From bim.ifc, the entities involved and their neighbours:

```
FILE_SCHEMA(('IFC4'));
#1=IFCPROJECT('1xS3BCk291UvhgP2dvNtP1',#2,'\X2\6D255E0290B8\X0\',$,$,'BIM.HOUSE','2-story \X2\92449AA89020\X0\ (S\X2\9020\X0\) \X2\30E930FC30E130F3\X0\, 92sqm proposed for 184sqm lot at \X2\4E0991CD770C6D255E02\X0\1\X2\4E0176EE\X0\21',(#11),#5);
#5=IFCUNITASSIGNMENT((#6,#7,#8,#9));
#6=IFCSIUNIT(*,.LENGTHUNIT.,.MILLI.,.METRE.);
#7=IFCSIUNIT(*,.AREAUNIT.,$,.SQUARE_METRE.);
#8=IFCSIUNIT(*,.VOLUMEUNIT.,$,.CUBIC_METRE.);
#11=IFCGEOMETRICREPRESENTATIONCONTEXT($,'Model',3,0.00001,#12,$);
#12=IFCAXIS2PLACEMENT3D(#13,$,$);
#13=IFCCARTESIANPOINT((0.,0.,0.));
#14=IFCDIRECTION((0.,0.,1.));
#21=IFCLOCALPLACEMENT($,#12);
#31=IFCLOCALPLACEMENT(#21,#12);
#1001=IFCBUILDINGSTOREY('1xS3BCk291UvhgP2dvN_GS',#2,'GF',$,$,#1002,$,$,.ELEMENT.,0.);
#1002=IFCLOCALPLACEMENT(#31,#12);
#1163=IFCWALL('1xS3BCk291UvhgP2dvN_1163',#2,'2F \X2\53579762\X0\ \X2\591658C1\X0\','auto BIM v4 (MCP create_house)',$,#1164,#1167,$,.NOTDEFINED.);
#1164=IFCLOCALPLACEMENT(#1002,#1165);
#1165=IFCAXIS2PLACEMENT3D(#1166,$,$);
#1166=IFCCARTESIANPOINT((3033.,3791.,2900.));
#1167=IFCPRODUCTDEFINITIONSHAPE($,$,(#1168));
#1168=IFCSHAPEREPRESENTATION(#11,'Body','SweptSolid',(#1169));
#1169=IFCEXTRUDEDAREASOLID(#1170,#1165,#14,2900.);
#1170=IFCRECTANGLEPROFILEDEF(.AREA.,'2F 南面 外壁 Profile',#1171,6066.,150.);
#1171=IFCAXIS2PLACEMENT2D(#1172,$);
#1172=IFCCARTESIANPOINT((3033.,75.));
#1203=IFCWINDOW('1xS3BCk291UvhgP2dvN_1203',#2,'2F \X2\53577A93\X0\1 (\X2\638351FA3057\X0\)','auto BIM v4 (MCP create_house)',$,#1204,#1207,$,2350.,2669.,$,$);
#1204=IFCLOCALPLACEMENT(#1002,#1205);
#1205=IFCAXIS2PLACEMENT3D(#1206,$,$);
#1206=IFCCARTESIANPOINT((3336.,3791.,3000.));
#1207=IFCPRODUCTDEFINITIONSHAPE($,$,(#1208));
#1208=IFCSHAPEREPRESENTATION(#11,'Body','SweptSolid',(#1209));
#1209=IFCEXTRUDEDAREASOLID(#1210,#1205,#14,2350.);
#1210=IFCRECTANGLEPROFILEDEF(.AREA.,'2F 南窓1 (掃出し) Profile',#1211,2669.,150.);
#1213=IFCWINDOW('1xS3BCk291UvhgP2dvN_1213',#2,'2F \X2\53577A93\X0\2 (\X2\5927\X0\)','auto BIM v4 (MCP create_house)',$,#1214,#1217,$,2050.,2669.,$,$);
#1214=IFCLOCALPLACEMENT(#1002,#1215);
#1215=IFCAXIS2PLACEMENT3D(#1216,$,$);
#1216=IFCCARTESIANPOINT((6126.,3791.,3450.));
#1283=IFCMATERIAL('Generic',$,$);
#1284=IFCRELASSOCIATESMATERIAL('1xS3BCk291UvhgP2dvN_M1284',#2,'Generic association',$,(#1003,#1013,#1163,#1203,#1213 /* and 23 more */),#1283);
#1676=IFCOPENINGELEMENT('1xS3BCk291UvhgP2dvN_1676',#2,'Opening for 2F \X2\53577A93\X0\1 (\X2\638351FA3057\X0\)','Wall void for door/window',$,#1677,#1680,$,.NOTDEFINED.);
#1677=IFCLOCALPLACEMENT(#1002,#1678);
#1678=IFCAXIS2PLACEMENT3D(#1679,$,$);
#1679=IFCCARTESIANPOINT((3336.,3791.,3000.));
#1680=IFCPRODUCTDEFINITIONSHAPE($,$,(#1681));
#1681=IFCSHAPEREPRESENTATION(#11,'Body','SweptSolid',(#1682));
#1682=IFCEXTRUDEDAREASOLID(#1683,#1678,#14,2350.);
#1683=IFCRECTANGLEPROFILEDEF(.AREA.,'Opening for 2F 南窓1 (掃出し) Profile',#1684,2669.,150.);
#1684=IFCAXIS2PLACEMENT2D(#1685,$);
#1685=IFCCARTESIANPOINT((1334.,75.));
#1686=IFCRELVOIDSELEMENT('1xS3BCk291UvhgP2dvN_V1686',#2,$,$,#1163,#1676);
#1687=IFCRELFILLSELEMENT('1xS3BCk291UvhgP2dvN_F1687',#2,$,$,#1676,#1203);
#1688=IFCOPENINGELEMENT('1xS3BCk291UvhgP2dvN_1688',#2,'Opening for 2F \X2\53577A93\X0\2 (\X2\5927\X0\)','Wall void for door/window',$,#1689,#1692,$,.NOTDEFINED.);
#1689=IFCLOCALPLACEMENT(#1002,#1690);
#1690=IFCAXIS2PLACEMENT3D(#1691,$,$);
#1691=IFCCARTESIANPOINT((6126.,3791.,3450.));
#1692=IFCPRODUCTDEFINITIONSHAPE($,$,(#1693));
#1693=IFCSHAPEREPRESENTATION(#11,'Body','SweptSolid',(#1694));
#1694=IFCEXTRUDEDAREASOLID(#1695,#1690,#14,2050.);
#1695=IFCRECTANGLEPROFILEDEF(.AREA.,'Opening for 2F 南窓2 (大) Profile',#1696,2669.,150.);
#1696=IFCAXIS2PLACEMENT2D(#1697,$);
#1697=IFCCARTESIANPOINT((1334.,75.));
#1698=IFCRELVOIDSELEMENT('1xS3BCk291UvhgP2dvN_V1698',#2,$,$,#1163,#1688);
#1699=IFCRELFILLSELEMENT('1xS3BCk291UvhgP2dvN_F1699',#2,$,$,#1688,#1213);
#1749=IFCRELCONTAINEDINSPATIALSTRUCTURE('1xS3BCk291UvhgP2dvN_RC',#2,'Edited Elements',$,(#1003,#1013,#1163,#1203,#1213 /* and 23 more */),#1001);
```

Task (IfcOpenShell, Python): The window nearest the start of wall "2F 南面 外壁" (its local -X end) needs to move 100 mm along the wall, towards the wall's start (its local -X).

```python
import ifcopenshell
import ifcopenshell.api.geometry
import ifcopenshell.util.placement
import ifcopenshell.util.unit

model = ifcopenshell.open("bim.ifc")
unit_scale = ifcopenshell.util.unit.calculate_unit_scale(model)

window = model.by_guid("1xS3BCk291UvhgP2dvN_1203")
opening = window.FillsVoids[0].RelatingOpeningElement
wall = opening.VoidsElements[0].RelatingBuildingElement

wall_matrix = ifcopenshell.util.placement.get_local_placement(wall.ObjectPlacement)
shift = wall_matrix[:3, 0] * -0.1 / unit_scale
before = ifcopenshell.util.placement.get_local_placement(window.ObjectPlacement)[:3, 3].copy()

# The window is not placed relative to its opening, so move both.
for product in (opening, window):
    matrix = ifcopenshell.util.placement.get_local_placement(product.ObjectPlacement)
    matrix[:3, 3] += shift
    ifcopenshell.api.geometry.edit_object_placement(model, product=product, matrix=matrix, is_si=False)

after = ifcopenshell.util.placement.get_local_placement(window.ObjectPlacement)[:3, 3]
print("window moved by", (after - before).round(3) + 0.0)

model.write("bim_updated.ifc")
```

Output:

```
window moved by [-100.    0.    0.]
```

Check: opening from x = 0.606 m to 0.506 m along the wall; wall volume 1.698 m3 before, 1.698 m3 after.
